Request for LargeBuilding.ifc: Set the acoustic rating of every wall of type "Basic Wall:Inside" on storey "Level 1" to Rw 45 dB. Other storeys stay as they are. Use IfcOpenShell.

First a look at what the model holds.

```python
import ifcopenshell
import ifcopenshell.util.element

model = ifcopenshell.open("LargeBuilding.ifc")
print(model.schema)
storey = next(s for s in model.by_type("IfcBuildingStorey") if s.Name == "Level 1")
walls = [e for e in ifcopenshell.util.element.get_decomposition(storey) if e.is_a("IfcWall")]
seen = {}
for e in walls:
    element_type = ifcopenshell.util.element.get_type(e)
    key = (element_type.Name if element_type != e and element_type else None, ifcopenshell.util.element.get_pset(e, "Pset_WallCommon", "AcousticRating"))
    seen[key] = seen.get(key, 0) + 1
for (name, value), count in sorted(seen.items(), key=str):
    print(count, "x", name, "|", value)
```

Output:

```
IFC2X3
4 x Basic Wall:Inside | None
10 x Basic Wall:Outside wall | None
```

```python
import ifcopenshell
import ifcopenshell.api.pset
import ifcopenshell.util.element

model = ifcopenshell.open("LargeBuilding.ifc")

storey = next(s for s in model.by_type("IfcBuildingStorey") if s.Name == "Level 1")
walls = [e for e in ifcopenshell.util.element.get_decomposition(storey) if e.is_a("IfcWall")]

count = 0
for e in walls:
    element_type = ifcopenshell.util.element.get_type(e)
    if element_type in (None, e) or element_type.Name != "Basic Wall:Inside":
        continue
    # add_pset returns the element's existing set when there is one.
    pset = ifcopenshell.api.pset.add_pset(model, product=e, name="Pset_WallCommon")
    ifcopenshell.api.pset.edit_pset(model, pset=pset, properties={"AcousticRating": "Rw 45 dB"})
    count += 1

print(count, "walls updated")

model.write("LargeBuilding_v2.ifc")
```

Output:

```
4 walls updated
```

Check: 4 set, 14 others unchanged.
